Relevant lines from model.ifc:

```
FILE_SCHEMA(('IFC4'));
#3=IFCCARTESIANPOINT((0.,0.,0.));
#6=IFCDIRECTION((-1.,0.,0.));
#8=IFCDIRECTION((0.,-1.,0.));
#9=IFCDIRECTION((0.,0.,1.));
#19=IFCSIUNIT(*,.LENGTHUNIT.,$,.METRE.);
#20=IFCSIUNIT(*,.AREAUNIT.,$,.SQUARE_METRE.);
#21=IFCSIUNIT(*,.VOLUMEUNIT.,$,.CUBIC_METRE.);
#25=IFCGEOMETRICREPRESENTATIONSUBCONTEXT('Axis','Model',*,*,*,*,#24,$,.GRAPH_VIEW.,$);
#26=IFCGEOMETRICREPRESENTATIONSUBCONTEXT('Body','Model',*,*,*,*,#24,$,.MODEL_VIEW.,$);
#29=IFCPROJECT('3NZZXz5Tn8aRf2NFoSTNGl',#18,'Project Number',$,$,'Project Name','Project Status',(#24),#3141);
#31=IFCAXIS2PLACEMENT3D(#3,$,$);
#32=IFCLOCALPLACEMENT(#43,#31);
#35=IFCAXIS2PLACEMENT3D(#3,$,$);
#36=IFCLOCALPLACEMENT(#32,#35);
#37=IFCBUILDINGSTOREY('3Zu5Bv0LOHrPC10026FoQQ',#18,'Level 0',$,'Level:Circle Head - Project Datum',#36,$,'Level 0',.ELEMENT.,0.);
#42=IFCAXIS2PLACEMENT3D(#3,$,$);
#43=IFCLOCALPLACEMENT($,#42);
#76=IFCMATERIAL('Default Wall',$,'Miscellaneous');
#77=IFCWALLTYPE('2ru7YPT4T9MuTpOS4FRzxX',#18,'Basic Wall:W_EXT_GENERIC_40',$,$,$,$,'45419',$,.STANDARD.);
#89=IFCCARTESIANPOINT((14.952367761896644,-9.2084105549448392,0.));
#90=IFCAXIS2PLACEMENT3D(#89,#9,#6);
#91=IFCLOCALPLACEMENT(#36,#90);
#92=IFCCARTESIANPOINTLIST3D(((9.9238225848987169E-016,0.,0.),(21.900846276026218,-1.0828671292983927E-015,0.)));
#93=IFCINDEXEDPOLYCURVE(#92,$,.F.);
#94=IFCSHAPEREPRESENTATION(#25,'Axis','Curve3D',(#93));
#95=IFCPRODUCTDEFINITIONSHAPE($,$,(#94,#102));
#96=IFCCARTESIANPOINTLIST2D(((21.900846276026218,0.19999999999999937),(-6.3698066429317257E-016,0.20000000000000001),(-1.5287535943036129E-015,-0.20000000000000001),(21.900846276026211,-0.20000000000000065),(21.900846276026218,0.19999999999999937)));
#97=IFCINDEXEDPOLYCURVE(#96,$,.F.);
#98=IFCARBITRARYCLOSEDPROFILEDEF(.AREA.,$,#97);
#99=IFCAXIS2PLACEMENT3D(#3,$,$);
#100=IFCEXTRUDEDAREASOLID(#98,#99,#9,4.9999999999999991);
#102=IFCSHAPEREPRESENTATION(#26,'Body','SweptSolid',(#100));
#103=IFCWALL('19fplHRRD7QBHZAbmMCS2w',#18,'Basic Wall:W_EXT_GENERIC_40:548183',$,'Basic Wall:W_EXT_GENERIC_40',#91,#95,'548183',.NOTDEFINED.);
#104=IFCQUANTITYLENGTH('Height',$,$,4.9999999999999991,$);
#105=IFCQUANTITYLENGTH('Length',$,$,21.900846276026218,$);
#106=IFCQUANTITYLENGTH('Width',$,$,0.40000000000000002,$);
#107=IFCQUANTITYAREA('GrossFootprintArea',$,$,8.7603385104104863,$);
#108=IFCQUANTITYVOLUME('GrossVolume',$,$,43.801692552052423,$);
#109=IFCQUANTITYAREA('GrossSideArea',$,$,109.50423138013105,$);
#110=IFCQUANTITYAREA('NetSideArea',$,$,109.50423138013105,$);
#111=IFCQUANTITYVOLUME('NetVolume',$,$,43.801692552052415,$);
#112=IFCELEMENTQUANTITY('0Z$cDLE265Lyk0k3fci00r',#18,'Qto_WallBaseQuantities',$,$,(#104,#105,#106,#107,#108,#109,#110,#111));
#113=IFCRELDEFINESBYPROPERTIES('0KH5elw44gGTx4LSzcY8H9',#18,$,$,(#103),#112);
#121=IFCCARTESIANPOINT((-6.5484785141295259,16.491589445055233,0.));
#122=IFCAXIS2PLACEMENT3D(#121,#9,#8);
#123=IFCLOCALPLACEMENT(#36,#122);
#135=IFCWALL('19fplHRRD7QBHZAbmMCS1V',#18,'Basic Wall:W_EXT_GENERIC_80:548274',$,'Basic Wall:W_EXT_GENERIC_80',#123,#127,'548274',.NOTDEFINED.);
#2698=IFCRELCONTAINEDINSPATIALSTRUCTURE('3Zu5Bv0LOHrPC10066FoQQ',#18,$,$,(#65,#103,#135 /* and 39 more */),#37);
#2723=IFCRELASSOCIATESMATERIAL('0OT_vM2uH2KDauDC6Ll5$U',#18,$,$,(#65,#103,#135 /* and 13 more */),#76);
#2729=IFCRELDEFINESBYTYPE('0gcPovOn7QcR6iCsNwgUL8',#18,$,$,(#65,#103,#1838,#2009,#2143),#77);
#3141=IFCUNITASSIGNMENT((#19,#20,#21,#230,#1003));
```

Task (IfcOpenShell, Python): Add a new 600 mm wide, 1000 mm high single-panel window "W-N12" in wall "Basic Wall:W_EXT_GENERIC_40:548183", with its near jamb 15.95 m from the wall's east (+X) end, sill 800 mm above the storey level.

```python
import numpy as np
import ifcopenshell
import ifcopenshell.api.feature
import ifcopenshell.api.geometry
import ifcopenshell.api.pset
import ifcopenshell.api.root
import ifcopenshell.api.spatial
import ifcopenshell.geom
import ifcopenshell.util.element
import ifcopenshell.util.placement
import ifcopenshell.util.representation
import ifcopenshell.util.shape
import ifcopenshell.util.unit

model = ifcopenshell.open("model.ifc")
unit_scale = ifcopenshell.util.unit.calculate_unit_scale(model)
area_scale = ifcopenshell.util.unit.calculate_unit_scale(model, "AREAUNIT")
volume_scale = ifcopenshell.util.unit.calculate_unit_scale(model, "VOLUMEUNIT")
settings = ifcopenshell.geom.settings()


def volume(element):
    """Net volume in cubic metres, openings subtracted."""
    shape = ifcopenshell.geom.create_shape(settings, element)
    return ifcopenshell.util.shape.get_volume(shape.geometry)


wall = model.by_guid("19fplHRRD7QBHZAbmMCS2w")
storey = ifcopenshell.util.element.get_container(wall, ifc_class="IfcBuildingStorey")
context = ifcopenshell.util.representation.get_context(model, "Model", "Body", "MODEL_VIEW")
before = volume(wall)

width, height, from_end, sill = 0.6, 1, 15.95, 0.8  # metres

# The wall runs along its own X axis, and the end named is its -X end.
wall_shape = ifcopenshell.geom.create_shape(settings, wall)
x, y, z = ifcopenshell.util.shape.get_vertices(wall_shape.geometry).T
start = x.min() + from_end
face, thickness = float(y.min()), float(y.max() - y.min())
wall_matrix = ifcopenshell.util.placement.get_local_placement(wall.ObjectPlacement)
level = ifcopenshell.util.placement.get_local_placement(storey.ObjectPlacement)[2, 3]


def in_wall(x, y):
    """Placement at x, y metres in the wall's axes, at sill height."""
    matrix = wall_matrix.copy()
    matrix[:, 3] = wall_matrix @ np.array([x / unit_scale, y / unit_scale, 0.0, 1.0])
    matrix[2, 3] = level + sill / unit_scale
    return matrix


# Opening: a box that overshoots both wall faces by 50 mm.
opening = ifcopenshell.api.root.create_entity(model, ifc_class="IfcOpeningElement", predefined_type="OPENING")
box = ifcopenshell.api.geometry.add_wall_representation(
    model, context=context, length=width, height=height, thickness=thickness + 0.1
)
ifcopenshell.api.geometry.assign_representation(model, product=opening, representation=box)
ifcopenshell.api.geometry.edit_object_placement(model, product=opening, matrix=in_wall(start, face - 0.05), is_si=False)
ifcopenshell.api.feature.add_feature(model, feature=opening, element=wall)

window = ifcopenshell.api.root.create_entity(model, ifc_class="IfcWindow", name="W-N12", predefined_type="WINDOW")
window.OverallWidth, window.OverallHeight = width / unit_scale, height / unit_scale
window.PartitioningType = "SINGLE_PANEL"
body = ifcopenshell.api.geometry.add_window_representation(
    model,
    context=context,
    overall_width=window.OverallWidth,
    overall_height=window.OverallHeight,
    partition_type="SINGLE_PANEL",
)
ifcopenshell.api.geometry.assign_representation(model, product=window, representation=body)
ifcopenshell.api.spatial.assign_container(model, products=[window], relating_structure=storey)
ifcopenshell.api.feature.add_filling(model, opening=opening, element=window)

# Centre the window in the wall's thickness.
ifcopenshell.api.geometry.edit_object_placement(model, product=window, matrix=in_wall(start, face), is_si=False)
window_shape = ifcopenshell.geom.create_shape(settings, window)
depth = ifcopenshell.util.shape.get_vertices(window_shape.geometry)[:, 1]
offset = face + thickness / 2 - (depth.min() + depth.max()) / 2
ifcopenshell.api.geometry.edit_object_placement(model, product=window, matrix=in_wall(start, offset), is_si=False)

after = volume(wall)

# Update the wall's stored quantities.
qto = model.by_id(ifcopenshell.util.element.get_pset(wall, "Qto_WallBaseQuantities", should_inherit=False)["id"])
ifcopenshell.api.pset.edit_qto(model, qto=qto, properties={
    "NetSideArea": after / thickness / area_scale,
    "NetVolume": after / volume_scale,
})

print(f"wall volume {before:.3f} -> {after:.3f} m3")

model.write("model_edited.ifc")
```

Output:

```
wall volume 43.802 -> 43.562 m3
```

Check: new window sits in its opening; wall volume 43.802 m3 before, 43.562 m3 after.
